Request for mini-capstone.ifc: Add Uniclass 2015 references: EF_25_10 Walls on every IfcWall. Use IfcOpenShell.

First a look at what the model holds.

```python
import ifcopenshell

model = ifcopenshell.open("mini-capstone.ifc")
print(model.schema)
print("classifications:", [c.Name for c in model.by_type("IfcClassification")])
for ifc_class in ("IfcDoor", "IfcRoof", "IfcStair", "IfcWall", "IfcWindow"):
    print(ifc_class, len(model.by_type(ifc_class)))
```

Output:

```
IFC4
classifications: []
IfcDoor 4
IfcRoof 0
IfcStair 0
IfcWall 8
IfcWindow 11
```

```python
import ifcopenshell
import ifcopenshell.api.classification

model = ifcopenshell.open("mini-capstone.ifc")

system = ifcopenshell.api.classification.add_classification(model, classification="Uniclass 2015")

codes = {
    "IfcWall": ("EF_25_10", "Walls"),
}
for ifc_class, (code, name) in codes.items():
    products = model.by_type(ifc_class)
    ifcopenshell.api.classification.add_reference(
        model, products=products, classification=system, identification=code, name=name
    )
    print(code, len(products))

model.write("mini-capstone_updated.ifc")
```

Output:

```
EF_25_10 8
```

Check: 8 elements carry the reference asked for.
